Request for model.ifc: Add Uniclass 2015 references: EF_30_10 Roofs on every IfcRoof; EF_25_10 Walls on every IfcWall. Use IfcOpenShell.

First a look at what the model holds.

```python
import ifcopenshell

model = ifcopenshell.open("model.ifc")
print(model.schema)
print("classifications:", [c.Name for c in model.by_type("IfcClassification")])
for ifc_class in ("IfcDoor", "IfcRoof", "IfcStair", "IfcWall", "IfcWindow"):
    print(ifc_class, len(model.by_type(ifc_class)))
```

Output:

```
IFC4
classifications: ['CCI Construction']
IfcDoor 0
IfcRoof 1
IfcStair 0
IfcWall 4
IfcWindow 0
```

```python
import ifcopenshell
import ifcopenshell.api.classification

model = ifcopenshell.open("model.ifc")

system = ifcopenshell.api.classification.add_classification(model, classification="Uniclass 2015")

codes = {
    "IfcRoof": ("EF_30_10", "Roofs"),
    "IfcWall": ("EF_25_10", "Walls"),
}
for ifc_class, (code, name) in codes.items():
    products = model.by_type(ifc_class)
    ifcopenshell.api.classification.add_reference(
        model, products=products, classification=system, identification=code, name=name
    )
    print(code, len(products))

model.write("model-out.ifc")
```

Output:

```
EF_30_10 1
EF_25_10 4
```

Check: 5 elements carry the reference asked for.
